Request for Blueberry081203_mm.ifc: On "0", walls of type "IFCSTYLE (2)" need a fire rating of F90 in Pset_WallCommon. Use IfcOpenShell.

First a look at what the model holds.

```python
import ifcopenshell
import ifcopenshell.util.element

model = ifcopenshell.open("Blueberry081203_mm.ifc")
print(model.schema)
storey = next(s for s in model.by_type("IfcBuildingStorey") if s.Name == "0")
walls = [e for e in ifcopenshell.util.element.get_decomposition(storey) if e.is_a("IfcWall")]
seen = {}
for e in walls:
    element_type = ifcopenshell.util.element.get_type(e)
    key = (element_type.Name if element_type != e and element_type else None, ifcopenshell.util.element.get_pset(e, "Pset_WallCommon", "FireRating"))
    seen[key] = seen.get(key, 0) + 1
for (name, value), count in sorted(seen.items(), key=str):
    print(count, "x", name, "|", value)
```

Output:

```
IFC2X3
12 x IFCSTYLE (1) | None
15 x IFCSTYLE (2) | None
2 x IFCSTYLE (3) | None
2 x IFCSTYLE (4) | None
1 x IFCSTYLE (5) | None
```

```python
import ifcopenshell
import ifcopenshell.api.pset
import ifcopenshell.util.element

model = ifcopenshell.open("Blueberry081203_mm.ifc")

storey = next(s for s in model.by_type("IfcBuildingStorey") if s.Name == "0")
walls = [e for e in ifcopenshell.util.element.get_decomposition(storey) if e.is_a("IfcWall")]

count = 0
for e in walls:
    element_type = ifcopenshell.util.element.get_type(e)
    if element_type in (None, e) or element_type.Name != "IFCSTYLE (2)":
        continue
    # add_pset returns the element's existing set when there is one.
    pset = ifcopenshell.api.pset.add_pset(model, product=e, name="Pset_WallCommon")
    ifcopenshell.api.pset.edit_pset(model, pset=pset, properties={"FireRating": "F90"})
    count += 1

print(count, "walls updated")

model.write("Blueberry081203_mm_edited.ifc")
```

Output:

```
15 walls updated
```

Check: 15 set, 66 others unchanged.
